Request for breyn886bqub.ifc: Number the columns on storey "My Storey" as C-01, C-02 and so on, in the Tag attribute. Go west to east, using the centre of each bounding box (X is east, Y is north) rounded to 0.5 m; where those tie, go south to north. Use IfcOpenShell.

First a look at what the model holds.

```python
import ifcopenshell
import ifcopenshell.util.element
import ifcopenshell.util.placement

model = ifcopenshell.open("breyn886bqub.ifc")
print(model.schema)
storey = next(s for s in model.by_type("IfcBuildingStorey") if s.Name == "My Storey")
columns = [e for e in ifcopenshell.util.element.get_decomposition(storey) if e.is_a("IfcColumn")]
for e in sorted(columns, key=lambda e: e.id()):
    origin = ifcopenshell.util.placement.get_local_placement(e.ObjectPlacement)[:3, 3]
    print(e.id(), e.Tag, e.Name, origin.round(2) + 0.0, sep=" | ")
```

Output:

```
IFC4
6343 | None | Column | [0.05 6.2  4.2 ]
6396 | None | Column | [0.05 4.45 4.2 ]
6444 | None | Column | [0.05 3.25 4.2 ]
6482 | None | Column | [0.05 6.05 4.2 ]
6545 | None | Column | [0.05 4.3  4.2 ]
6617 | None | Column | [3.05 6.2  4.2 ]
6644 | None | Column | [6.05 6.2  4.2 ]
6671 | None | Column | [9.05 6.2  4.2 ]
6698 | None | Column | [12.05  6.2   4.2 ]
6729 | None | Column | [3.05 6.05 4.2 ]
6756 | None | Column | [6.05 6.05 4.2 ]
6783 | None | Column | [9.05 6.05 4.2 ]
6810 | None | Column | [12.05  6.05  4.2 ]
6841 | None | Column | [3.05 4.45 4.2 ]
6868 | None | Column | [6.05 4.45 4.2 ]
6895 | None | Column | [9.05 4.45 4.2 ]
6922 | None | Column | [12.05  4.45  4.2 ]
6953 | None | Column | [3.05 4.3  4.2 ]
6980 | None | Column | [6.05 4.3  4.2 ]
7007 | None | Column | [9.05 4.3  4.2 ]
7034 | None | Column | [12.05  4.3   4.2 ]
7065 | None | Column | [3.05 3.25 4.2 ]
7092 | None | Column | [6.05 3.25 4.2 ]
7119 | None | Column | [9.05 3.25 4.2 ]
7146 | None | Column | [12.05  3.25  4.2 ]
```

```python
import ifcopenshell
import ifcopenshell.geom
import ifcopenshell.util.element
import ifcopenshell.util.shape

model = ifcopenshell.open("breyn886bqub.ifc")
settings = ifcopenshell.geom.settings()
settings.set("use-world-coords", True)


def centre(element):
    shape = ifcopenshell.geom.create_shape(settings, element)
    return ifcopenshell.util.shape.get_bbox_centroid(shape.geometry)


storey = next(s for s in model.by_type("IfcBuildingStorey") if s.Name == "My Storey")
columns = [e for e in ifcopenshell.util.element.get_decomposition(storey) if e.is_a("IfcColumn")]

# Insertion points can sit at a corner or the storey origin, so sort by the geometry (in metres).
centres = {e: centre(e) for e in columns}
columns.sort(key=lambda e: (round(centres[e][0] / 0.5), centres[e][1]))

for i, e in enumerate(columns, start=1):
    number = f"C-{i:02d}"
    e.Tag = number
    print(e.id(), number)

model.write("breyn886bqub_rev.ifc")
```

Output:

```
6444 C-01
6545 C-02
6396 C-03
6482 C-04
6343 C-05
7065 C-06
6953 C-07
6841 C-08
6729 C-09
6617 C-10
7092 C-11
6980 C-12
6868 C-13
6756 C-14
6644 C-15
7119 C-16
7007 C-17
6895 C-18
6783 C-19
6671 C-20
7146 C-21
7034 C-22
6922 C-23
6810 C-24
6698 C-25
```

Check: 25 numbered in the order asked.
